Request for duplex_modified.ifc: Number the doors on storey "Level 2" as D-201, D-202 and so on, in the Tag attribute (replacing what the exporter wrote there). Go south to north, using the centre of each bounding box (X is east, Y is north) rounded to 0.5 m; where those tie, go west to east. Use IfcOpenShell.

First a look at what the model holds.

```python
import ifcopenshell
import ifcopenshell.util.element
import ifcopenshell.util.placement

model = ifcopenshell.open("duplex_modified.ifc")
print(model.schema)
storey = next(s for s in model.by_type("IfcBuildingStorey") if s.Name == "Level 2")
doors = [e for e in ifcopenshell.util.element.get_decomposition(storey) if e.is_a("IfcDoor")]
for e in sorted(doors, key=lambda e: e.id()):
    origin = ifcopenshell.util.placement.get_local_placement(e.ObjectPlacement)[:3, 3]
    print(e.id(), e.Tag, e.Name, origin.round(2) + 0.0, sep=" | ")
```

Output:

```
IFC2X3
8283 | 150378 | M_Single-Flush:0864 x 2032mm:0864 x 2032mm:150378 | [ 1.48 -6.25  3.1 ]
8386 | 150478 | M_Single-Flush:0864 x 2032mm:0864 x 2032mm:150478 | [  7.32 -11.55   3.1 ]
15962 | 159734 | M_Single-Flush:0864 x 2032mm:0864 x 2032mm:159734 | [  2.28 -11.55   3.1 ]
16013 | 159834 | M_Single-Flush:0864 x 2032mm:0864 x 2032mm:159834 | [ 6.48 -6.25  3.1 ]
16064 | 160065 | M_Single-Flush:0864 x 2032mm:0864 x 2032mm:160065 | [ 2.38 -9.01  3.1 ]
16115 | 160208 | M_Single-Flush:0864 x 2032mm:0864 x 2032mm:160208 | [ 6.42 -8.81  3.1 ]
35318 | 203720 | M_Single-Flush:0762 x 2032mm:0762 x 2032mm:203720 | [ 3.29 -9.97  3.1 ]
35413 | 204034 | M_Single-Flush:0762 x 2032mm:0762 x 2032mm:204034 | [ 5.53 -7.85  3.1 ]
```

```python
import ifcopenshell
import ifcopenshell.geom
import ifcopenshell.util.element
import ifcopenshell.util.shape

model = ifcopenshell.open("duplex_modified.ifc")
settings = ifcopenshell.geom.settings()
settings.set("use-world-coords", True)


def centre(element):
    shape = ifcopenshell.geom.create_shape(settings, element)
    return ifcopenshell.util.shape.get_bbox_centroid(shape.geometry)


storey = next(s for s in model.by_type("IfcBuildingStorey") if s.Name == "Level 2")
doors = [e for e in ifcopenshell.util.element.get_decomposition(storey) if e.is_a("IfcDoor")]

# Insertion points can sit at a corner or the storey origin, so sort by the geometry (in metres).
centres = {e: centre(e) for e in doors}
doors.sort(key=lambda e: (round(centres[e][1] / 0.5), centres[e][0]))

for i, e in enumerate(doors, start=1):
    number = f"D-2{i:02d}"
    e.Tag = number
    print(e.id(), number)

model.write("duplex_modified_v2.ifc")
```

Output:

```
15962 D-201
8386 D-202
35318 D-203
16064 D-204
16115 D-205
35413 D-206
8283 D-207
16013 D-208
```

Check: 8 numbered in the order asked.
